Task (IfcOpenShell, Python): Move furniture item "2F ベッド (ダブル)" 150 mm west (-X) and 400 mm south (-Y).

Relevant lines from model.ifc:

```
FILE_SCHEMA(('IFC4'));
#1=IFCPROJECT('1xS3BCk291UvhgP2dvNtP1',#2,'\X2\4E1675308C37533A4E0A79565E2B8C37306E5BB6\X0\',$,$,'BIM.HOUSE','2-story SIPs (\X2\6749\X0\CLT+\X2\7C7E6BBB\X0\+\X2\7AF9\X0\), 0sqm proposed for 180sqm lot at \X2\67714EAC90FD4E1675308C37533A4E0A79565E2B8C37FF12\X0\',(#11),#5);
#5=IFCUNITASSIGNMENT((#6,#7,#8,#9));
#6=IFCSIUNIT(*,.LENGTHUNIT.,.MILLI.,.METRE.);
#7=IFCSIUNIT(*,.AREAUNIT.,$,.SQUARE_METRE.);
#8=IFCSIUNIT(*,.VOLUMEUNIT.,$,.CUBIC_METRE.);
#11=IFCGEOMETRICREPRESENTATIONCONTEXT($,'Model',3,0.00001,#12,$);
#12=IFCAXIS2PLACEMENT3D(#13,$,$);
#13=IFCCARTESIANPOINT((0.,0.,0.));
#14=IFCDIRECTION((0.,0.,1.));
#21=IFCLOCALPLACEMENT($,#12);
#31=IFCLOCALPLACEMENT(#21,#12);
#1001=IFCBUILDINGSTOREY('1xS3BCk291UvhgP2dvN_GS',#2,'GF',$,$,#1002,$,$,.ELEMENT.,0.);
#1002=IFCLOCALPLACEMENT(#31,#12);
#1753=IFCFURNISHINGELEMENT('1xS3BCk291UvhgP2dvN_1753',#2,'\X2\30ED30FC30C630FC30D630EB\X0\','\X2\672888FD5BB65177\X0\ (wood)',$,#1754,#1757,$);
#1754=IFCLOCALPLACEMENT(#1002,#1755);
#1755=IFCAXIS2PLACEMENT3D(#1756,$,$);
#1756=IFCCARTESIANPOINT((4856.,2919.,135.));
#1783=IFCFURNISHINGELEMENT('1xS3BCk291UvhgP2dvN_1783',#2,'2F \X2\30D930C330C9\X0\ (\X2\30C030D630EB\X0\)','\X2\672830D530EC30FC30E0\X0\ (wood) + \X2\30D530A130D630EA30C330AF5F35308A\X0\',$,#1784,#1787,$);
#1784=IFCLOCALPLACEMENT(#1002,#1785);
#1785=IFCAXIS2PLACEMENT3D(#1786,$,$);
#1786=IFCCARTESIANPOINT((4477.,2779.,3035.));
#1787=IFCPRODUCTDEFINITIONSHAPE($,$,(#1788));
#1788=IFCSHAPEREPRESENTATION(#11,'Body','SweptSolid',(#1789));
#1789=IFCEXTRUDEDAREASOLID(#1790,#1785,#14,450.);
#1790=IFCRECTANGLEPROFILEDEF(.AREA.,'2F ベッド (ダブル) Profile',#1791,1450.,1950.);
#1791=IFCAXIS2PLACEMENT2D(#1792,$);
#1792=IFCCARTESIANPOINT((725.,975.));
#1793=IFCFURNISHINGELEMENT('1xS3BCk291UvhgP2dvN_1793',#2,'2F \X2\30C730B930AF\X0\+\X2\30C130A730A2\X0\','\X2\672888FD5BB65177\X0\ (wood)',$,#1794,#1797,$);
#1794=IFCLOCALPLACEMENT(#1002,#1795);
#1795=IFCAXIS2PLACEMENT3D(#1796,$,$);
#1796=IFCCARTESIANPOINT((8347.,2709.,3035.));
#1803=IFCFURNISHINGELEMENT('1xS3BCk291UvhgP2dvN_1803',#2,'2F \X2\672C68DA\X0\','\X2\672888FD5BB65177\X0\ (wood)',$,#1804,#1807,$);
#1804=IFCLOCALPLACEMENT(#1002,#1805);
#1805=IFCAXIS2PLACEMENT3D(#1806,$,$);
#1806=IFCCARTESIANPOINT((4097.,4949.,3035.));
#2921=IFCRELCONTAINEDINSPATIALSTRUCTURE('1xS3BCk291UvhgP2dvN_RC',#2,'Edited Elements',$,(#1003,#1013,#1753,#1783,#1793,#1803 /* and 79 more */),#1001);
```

```python
import ifcopenshell
import ifcopenshell.api.geometry
import ifcopenshell.util.placement

model = ifcopenshell.open("model.ifc")

item = model.by_guid("1xS3BCk291UvhgP2dvN_1783")
matrix = ifcopenshell.util.placement.get_local_placement(item.ObjectPlacement)
matrix[0, 3] -= 150.0
matrix[1, 3] -= 400.0
ifcopenshell.api.geometry.edit_object_placement(model, product=item, matrix=matrix, is_si=False)

print(ifcopenshell.util.placement.get_local_placement(item.ObjectPlacement).round(3) + 0.0)

model.write("model_rev.ifc")
```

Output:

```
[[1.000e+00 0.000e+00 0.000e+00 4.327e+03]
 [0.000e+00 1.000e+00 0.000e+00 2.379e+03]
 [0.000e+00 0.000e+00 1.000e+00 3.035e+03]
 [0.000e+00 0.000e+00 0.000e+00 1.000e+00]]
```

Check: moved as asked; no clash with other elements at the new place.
